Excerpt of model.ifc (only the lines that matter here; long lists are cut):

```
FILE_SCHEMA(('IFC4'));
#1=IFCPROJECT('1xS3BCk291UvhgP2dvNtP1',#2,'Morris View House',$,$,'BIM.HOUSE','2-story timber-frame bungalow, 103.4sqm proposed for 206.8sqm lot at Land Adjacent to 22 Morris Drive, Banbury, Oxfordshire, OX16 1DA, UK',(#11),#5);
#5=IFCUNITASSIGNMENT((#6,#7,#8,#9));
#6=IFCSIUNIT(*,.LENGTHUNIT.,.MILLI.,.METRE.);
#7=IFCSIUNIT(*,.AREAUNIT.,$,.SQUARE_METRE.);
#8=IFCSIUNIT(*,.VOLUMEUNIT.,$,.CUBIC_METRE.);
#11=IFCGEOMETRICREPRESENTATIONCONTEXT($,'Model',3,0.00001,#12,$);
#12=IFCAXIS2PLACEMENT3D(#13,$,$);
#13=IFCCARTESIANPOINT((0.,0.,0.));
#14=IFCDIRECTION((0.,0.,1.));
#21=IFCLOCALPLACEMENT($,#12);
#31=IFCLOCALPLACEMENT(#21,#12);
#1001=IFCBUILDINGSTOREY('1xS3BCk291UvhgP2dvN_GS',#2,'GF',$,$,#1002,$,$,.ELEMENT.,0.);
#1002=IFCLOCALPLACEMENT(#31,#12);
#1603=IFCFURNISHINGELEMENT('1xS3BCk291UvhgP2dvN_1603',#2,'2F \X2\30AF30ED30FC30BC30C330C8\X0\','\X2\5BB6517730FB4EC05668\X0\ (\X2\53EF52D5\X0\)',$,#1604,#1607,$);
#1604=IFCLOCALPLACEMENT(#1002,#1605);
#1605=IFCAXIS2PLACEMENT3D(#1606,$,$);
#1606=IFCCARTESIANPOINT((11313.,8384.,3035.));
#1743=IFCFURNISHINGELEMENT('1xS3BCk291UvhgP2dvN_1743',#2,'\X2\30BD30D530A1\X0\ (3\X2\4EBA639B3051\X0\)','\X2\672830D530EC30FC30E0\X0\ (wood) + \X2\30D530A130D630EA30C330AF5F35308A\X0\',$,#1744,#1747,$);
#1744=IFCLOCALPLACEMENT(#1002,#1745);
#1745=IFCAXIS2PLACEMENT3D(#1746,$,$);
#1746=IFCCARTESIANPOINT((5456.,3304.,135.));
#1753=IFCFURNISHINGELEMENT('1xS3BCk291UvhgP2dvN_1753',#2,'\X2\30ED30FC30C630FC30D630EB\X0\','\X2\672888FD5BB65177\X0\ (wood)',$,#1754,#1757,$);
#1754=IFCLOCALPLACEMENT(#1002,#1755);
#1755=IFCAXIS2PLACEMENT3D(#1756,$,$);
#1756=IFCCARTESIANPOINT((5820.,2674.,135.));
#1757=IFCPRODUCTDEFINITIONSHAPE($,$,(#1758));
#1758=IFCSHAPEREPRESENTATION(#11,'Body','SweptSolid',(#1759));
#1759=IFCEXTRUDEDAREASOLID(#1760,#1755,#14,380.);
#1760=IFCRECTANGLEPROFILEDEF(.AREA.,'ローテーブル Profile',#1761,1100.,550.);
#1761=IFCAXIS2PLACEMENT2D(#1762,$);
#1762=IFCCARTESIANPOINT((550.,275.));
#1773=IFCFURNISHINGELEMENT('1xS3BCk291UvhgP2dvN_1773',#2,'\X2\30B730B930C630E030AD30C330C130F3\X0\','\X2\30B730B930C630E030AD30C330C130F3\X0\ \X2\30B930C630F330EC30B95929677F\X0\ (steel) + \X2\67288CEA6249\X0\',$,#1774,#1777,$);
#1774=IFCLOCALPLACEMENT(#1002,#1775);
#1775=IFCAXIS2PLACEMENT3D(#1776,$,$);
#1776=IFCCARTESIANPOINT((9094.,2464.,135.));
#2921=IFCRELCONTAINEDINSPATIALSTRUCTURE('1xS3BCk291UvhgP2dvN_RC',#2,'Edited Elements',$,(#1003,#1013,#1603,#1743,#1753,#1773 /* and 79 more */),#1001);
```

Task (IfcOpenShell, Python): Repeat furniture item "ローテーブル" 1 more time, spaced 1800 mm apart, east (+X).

```python
import numpy as np
import ifcopenshell
import ifcopenshell.api.geometry
import ifcopenshell.api.root
import ifcopenshell.util.element
import ifcopenshell.util.placement
import ifcopenshell.util.unit

model = ifcopenshell.open("model.ifc")
unit_scale = ifcopenshell.util.unit.calculate_unit_scale(model)


def reuse_history(source, copy):
    """copy_class also copies each property set's owner history, people and application; keep the originals."""
    for rel in copy.IsDefinedBy:
        if rel.is_a("IfcRelDefinesByProperties") and (history := rel.RelatingPropertyDefinition.OwnerHistory):
            rel.RelatingPropertyDefinition.OwnerHistory = source.OwnerHistory
            ifcopenshell.util.element.remove_deep2(model, history)


source = model.by_guid("1xS3BCk291UvhgP2dvN_1753")
base = ifcopenshell.util.placement.get_local_placement(source.ObjectPlacement)
step = np.array([1.0, 0.0, 0.0]) * 1.8 / unit_scale

for i in range(1, 2):
    copy = ifcopenshell.api.root.copy_class(model, product=source)
    copy.Representation = ifcopenshell.util.element.copy_deep(
        model, source.Representation, exclude=["IfcGeometricRepresentationContext", "IfcRepresentationMap"]
    )
    reuse_history(source, copy)
    matrix = base.copy()
    matrix[:3, 3] += i * step
    print("added at", matrix[:3, 3].round(3) + 0.0)
    ifcopenshell.api.geometry.edit_object_placement(model, product=copy, matrix=matrix, is_si=False)

model.write("model_v2.ifc")
```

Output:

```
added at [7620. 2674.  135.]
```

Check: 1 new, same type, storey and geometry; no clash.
